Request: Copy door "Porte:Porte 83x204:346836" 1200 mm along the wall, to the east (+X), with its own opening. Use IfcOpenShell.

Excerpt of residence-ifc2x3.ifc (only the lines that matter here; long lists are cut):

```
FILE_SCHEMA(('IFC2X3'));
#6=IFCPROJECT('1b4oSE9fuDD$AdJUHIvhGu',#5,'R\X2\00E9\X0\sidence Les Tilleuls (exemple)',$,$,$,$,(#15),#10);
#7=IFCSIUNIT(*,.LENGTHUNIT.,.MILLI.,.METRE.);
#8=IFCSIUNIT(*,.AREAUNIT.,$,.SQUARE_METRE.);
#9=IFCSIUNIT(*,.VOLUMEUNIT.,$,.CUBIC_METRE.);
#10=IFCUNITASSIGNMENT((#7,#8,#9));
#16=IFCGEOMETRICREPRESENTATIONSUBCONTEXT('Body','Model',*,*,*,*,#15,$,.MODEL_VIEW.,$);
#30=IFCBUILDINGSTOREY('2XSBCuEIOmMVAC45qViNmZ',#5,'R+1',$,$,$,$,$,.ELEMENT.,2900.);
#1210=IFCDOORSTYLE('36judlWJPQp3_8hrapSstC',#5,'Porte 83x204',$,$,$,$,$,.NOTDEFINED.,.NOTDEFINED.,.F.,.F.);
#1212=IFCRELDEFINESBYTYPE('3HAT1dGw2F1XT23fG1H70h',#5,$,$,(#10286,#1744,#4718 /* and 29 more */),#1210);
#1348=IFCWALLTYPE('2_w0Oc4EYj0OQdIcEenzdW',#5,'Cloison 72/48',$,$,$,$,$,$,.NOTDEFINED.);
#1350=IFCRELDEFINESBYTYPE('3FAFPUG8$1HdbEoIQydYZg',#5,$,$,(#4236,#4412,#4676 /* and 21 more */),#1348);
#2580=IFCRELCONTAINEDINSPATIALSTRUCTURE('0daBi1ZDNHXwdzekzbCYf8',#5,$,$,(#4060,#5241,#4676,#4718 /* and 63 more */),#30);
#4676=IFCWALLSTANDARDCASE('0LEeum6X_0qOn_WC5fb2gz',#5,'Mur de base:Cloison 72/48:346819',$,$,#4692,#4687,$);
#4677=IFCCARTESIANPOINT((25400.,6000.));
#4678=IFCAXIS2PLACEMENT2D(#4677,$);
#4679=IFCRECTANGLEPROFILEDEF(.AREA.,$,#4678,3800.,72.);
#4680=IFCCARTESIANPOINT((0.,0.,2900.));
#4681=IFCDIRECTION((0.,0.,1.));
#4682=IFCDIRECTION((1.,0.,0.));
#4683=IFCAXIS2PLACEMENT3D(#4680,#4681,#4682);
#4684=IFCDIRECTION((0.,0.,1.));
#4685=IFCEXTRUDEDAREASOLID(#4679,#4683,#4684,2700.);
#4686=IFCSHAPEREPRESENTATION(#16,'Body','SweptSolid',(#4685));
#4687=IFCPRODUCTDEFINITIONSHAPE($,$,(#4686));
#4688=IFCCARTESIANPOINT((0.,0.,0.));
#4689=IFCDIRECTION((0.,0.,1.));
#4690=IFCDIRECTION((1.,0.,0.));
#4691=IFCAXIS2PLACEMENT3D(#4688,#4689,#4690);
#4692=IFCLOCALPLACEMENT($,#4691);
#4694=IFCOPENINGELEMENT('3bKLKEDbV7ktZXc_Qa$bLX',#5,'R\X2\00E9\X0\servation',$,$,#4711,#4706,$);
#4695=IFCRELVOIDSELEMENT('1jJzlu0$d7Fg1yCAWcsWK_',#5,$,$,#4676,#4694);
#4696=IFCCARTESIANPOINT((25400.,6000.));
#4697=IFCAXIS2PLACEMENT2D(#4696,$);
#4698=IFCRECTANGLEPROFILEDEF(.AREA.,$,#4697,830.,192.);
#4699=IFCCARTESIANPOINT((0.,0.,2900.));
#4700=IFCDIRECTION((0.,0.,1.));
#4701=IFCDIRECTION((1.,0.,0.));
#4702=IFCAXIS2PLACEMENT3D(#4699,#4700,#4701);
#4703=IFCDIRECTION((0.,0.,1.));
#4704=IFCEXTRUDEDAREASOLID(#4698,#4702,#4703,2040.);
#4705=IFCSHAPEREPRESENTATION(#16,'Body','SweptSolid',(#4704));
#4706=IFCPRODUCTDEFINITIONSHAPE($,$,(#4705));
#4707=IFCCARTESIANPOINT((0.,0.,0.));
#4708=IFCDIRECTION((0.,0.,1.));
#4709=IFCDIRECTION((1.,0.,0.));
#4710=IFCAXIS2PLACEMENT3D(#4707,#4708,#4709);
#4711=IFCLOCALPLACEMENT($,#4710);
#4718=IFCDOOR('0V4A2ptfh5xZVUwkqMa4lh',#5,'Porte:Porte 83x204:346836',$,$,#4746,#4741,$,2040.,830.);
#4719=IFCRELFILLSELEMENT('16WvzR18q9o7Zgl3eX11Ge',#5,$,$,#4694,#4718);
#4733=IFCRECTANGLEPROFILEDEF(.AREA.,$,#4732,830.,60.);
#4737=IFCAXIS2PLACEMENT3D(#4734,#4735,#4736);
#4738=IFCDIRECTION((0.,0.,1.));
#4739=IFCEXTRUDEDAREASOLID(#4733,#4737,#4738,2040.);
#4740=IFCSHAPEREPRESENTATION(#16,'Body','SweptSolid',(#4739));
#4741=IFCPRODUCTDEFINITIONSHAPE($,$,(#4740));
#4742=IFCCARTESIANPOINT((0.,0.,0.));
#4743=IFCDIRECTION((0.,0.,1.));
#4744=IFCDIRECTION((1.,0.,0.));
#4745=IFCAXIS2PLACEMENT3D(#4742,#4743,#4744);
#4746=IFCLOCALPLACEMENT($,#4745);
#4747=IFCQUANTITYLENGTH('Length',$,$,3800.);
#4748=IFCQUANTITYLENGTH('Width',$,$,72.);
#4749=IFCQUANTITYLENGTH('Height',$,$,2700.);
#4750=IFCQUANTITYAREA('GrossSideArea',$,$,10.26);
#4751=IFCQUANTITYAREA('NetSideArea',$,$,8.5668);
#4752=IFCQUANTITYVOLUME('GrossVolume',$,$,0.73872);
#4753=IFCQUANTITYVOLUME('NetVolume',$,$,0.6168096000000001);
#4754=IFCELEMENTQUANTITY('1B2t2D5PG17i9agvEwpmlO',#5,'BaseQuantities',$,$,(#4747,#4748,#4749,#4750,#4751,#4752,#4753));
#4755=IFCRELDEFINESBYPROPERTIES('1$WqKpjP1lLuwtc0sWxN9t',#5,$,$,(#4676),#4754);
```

```python
import ifcopenshell
import ifcopenshell.api.feature
import ifcopenshell.api.geometry
import ifcopenshell.api.pset
import ifcopenshell.api.root
import ifcopenshell.geom
import ifcopenshell.util.element
import ifcopenshell.util.placement
import ifcopenshell.util.shape
import ifcopenshell.util.unit

model = ifcopenshell.open("residence-ifc2x3.ifc")
unit_scale = ifcopenshell.util.unit.calculate_unit_scale(model)
area_scale = ifcopenshell.util.unit.calculate_unit_scale(model, "AREAUNIT")
volume_scale = ifcopenshell.util.unit.calculate_unit_scale(model, "VOLUMEUNIT")
settings = ifcopenshell.geom.settings()


def volume(element):
    """Net volume in cubic metres, openings subtracted."""
    shape = ifcopenshell.geom.create_shape(settings, element)
    return ifcopenshell.util.shape.get_volume(shape.geometry)


def reuse_history(source, copy):
    """copy_class also copies each property set's owner history, people and application; keep the originals."""
    for rel in copy.IsDefinedBy:
        if rel.is_a("IfcRelDefinesByProperties") and (history := rel.RelatingPropertyDefinition.OwnerHistory):
            rel.RelatingPropertyDefinition.OwnerHistory = source.OwnerHistory
            ifcopenshell.util.element.remove_deep2(model, history)


door = model.by_guid("0V4A2ptfh5xZVUwkqMa4lh")
opening = door.FillsVoids[0].RelatingOpeningElement
wall = opening.VoidsElements[0].RelatingBuildingElement
before = volume(wall)
shift = ifcopenshell.util.placement.get_local_placement(wall.ObjectPlacement)[:3, 0] * 1.2 / unit_scale

# copy_class copies the void relationship, type, container and properties, but no geometry.
new_opening = ifcopenshell.api.root.copy_class(model, product=opening)
new_opening.Representation = ifcopenshell.util.element.copy_deep(
    model, opening.Representation, exclude=["IfcGeometricRepresentationContext", "IfcRepresentationMap"]
)
reuse_history(opening, new_opening)
new_door = ifcopenshell.api.root.copy_class(model, product=door)
new_door.Representation = ifcopenshell.util.element.copy_deep(
    model, door.Representation, exclude=["IfcGeometricRepresentationContext", "IfcRepresentationMap"]
)
new_door.Name = "Porte:Porte 83x204"
reuse_history(door, new_door)
fills = ifcopenshell.api.feature.add_filling(model, opening=new_opening, element=new_door)
fills.OwnerHistory = new_door.OwnerHistory  # required in IFC2X3

for old, new in ((opening, new_opening), (door, new_door)):
    matrix = ifcopenshell.util.placement.get_local_placement(old.ObjectPlacement)
    matrix[:3, 3] += shift
    ifcopenshell.api.geometry.edit_object_placement(model, product=new, matrix=matrix, is_si=False)

after = volume(wall)
thickness = 0.072  # wall thickness in metres

# Update the wall's stored quantities.
qto = model.by_id(ifcopenshell.util.element.get_pset(wall, "BaseQuantities", should_inherit=False)["id"])
ifcopenshell.api.pset.edit_qto(model, qto=qto, properties={
    "NetSideArea": after / thickness / area_scale,
    "NetVolume": after / volume_scale,
})

print(f"wall volume {before:.3f} -> {after:.3f} m3")

model.write("residence-ifc2x3_edited.ifc")
```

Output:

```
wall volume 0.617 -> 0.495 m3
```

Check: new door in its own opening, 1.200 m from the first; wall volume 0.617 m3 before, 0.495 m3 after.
